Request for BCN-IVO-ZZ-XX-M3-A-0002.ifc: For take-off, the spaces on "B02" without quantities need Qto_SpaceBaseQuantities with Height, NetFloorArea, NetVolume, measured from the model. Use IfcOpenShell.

First a look at what the model holds.

```python
import ifcopenshell
import ifcopenshell.util.element
import ifcopenshell.util.unit

model = ifcopenshell.open("BCN-IVO-ZZ-XX-M3-A-0002.ifc")
print(model.schema)
for unit_type in ("LENGTHUNIT", "AREAUNIT", "VOLUMEUNIT"):
    print(unit_type, ifcopenshell.util.unit.calculate_unit_scale(model, unit_type))
storey = next(s for s in model.by_type("IfcBuildingStorey") if s.Name == "B02")
spaces = [e for e in ifcopenshell.util.element.get_decomposition(storey) if e.is_a("IfcSpace")]
for e in sorted(spaces, key=lambda e: e.id()):
    print(e.id(), e.is_a(), e.Name, list(ifcopenshell.util.element.get_psets(e, qtos_only=True)), sep=" | ")
```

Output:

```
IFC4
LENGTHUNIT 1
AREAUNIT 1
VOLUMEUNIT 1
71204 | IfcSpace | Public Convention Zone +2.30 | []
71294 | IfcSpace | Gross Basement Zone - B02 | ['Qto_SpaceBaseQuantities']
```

```python
import ifcopenshell
import ifcopenshell.api.pset
import ifcopenshell.geom
import ifcopenshell.util.element
import ifcopenshell.util.shape
import ifcopenshell.util.unit

model = ifcopenshell.open("BCN-IVO-ZZ-XX-M3-A-0002.ifc")
unit_scale = ifcopenshell.util.unit.calculate_unit_scale(model)
area_scale = ifcopenshell.util.unit.calculate_unit_scale(model, "AREAUNIT")
volume_scale = ifcopenshell.util.unit.calculate_unit_scale(model, "VOLUMEUNIT")
settings = ifcopenshell.geom.settings()

storey = next(s for s in model.by_type("IfcBuildingStorey") if s.Name == "B02")
spaces = [e for e in ifcopenshell.util.element.get_decomposition(storey) if e.is_a("IfcSpace")]

for e in sorted(spaces, key=lambda e: e.id()):
    if ifcopenshell.util.element.get_psets(e, qtos_only=True, should_inherit=False):
        continue
    # Geometry comes back in metres, in the element's own axes.
    shape = ifcopenshell.geom.create_shape(settings, e)
    values = {
        "Height": ifcopenshell.util.shape.get_z(shape.geometry) / unit_scale,
        "NetFloorArea": ifcopenshell.util.shape.get_footprint_area(shape.geometry) / area_scale,
        "NetVolume": ifcopenshell.util.shape.get_volume(shape.geometry) / volume_scale,
    }
    qto = ifcopenshell.api.pset.add_qto(model, product=e, name="Qto_SpaceBaseQuantities")
    ifcopenshell.api.pset.edit_qto(model, qto=qto, properties=values)
    print(e.id(), {k: round(v, 3) for k, v in values.items()})

model.write("BCN-IVO-ZZ-XX-M3-A-0002_updated.ifc")
```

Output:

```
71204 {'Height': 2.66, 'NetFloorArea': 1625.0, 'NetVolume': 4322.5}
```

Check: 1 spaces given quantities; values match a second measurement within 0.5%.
